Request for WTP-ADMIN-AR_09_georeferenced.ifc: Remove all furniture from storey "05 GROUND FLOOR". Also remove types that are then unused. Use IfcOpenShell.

First a look at what the model holds.

```python
import ifcopenshell
import ifcopenshell.util.element

model = ifcopenshell.open("WTP-ADMIN-AR_09_georeferenced.ifc")
print(model.schema)
storey = next(s for s in model.by_type("IfcBuildingStorey") if s.Name == "05 GROUND FLOOR")
furniture = [e for e in ifcopenshell.util.element.get_decomposition(storey) if e.is_a("IfcFurnishingElement")]
seen = {}
for e in furniture:
    element_type = ifcopenshell.util.element.get_type(e)
    name = element_type.Name if element_type not in (None, e) else None
    seen[name] = seen.get(name, 0) + 1
for name, count in sorted(seen.items(), key=str):
    print(count, "x", name)
```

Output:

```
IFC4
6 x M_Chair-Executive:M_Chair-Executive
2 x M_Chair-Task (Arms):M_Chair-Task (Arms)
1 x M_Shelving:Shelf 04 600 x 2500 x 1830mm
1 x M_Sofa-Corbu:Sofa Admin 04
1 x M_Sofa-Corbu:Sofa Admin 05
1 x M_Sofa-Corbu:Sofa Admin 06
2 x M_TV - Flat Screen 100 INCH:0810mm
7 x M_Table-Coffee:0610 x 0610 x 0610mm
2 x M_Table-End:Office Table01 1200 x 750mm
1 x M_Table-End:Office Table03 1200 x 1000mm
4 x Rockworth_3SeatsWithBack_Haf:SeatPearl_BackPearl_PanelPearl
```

```python
import ifcopenshell
import ifcopenshell.api.root
import ifcopenshell.util.element

model = ifcopenshell.open("WTP-ADMIN-AR_09_georeferenced.ifc")

storey = next(s for s in model.by_type("IfcBuildingStorey") if s.Name == "05 GROUND FLOOR")
furniture = [e for e in ifcopenshell.util.element.get_decomposition(storey) if e.is_a("IfcFurnishingElement")]
types = {ifcopenshell.util.element.get_type(e) for e in furniture} - {None, *furniture}

for e in furniture:
    ifcopenshell.api.root.remove_product(model, product=e)
print(len(furniture), "removed")

unused = [t for t in types if not ifcopenshell.util.element.get_types(t)]
for t in unused:
    ifcopenshell.api.root.remove_product(model, product=t)
print(len(unused), "unused types removed")

model.write("WTP-ADMIN-AR_09_georeferenced-out.ifc")
```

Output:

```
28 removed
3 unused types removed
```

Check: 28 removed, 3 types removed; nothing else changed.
